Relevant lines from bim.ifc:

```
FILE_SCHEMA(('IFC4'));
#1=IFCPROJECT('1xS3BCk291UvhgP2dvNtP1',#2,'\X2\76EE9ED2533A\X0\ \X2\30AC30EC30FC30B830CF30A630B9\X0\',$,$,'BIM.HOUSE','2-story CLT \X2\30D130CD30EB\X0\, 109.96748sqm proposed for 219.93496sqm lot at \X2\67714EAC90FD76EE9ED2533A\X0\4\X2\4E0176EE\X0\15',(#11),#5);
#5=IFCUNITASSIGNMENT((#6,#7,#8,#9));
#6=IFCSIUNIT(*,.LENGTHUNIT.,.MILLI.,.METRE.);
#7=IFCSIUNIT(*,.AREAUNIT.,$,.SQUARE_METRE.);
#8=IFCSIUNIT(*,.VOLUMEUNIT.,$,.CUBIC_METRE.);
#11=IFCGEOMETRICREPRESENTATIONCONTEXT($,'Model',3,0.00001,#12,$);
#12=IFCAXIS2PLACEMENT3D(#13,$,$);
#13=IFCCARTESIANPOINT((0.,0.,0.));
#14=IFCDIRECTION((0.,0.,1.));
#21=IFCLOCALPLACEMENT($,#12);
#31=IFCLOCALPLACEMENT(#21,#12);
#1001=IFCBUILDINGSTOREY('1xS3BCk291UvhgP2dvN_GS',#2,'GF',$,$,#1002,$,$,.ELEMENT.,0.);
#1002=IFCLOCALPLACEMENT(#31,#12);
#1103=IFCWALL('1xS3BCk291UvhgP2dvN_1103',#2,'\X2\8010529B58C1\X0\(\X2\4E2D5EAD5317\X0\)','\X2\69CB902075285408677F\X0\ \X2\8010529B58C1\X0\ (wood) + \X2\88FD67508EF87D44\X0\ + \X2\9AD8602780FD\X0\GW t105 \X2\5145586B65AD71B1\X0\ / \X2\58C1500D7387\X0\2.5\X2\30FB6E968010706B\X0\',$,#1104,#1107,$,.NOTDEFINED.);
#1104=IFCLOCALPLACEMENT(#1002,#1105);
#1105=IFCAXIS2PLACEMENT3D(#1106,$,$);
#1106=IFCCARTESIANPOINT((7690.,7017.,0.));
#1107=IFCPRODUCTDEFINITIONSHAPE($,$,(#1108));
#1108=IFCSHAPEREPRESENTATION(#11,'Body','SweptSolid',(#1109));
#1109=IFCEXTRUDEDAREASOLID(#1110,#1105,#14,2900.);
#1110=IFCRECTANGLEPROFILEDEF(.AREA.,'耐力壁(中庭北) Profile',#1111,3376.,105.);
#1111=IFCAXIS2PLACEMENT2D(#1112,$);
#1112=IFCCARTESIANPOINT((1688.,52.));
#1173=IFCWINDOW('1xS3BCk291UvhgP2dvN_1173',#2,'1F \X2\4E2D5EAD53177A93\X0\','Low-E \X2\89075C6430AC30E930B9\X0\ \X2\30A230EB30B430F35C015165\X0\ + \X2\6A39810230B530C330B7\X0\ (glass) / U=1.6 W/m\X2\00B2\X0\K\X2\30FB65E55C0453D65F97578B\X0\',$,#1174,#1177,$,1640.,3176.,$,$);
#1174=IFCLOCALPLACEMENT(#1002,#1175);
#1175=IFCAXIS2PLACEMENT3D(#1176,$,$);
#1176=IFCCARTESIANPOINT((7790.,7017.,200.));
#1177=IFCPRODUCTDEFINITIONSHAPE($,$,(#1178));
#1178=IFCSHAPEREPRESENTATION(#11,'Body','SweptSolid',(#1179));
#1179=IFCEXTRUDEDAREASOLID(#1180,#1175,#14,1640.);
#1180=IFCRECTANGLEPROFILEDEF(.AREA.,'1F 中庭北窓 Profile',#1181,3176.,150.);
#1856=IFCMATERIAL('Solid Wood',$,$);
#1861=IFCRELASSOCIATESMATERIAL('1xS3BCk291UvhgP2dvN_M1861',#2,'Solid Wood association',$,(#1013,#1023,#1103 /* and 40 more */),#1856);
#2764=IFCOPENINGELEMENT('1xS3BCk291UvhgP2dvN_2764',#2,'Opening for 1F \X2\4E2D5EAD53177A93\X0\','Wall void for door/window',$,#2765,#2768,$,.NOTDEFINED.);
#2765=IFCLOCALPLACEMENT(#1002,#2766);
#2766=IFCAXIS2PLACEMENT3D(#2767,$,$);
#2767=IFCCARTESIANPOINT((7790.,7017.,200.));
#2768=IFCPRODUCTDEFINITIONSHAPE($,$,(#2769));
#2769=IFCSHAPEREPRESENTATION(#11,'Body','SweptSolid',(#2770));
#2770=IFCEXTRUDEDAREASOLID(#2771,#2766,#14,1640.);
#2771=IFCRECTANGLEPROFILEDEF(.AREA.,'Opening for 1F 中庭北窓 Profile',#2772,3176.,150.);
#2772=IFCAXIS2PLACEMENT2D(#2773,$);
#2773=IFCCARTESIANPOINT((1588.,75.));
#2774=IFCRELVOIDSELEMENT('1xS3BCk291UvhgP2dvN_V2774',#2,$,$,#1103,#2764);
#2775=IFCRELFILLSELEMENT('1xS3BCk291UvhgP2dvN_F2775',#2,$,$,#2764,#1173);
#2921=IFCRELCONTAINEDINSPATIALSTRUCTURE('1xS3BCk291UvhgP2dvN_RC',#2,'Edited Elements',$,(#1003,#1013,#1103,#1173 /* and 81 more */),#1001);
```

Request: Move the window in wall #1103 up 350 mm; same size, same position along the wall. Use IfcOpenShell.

```python
import numpy as np
import ifcopenshell
import ifcopenshell.api.geometry
import ifcopenshell.util.placement
import ifcopenshell.util.unit

model = ifcopenshell.open("bim.ifc")
unit_scale = ifcopenshell.util.unit.calculate_unit_scale(model)

window = model.by_guid("1xS3BCk291UvhgP2dvN_1173")
opening = window.FillsVoids[0].RelatingOpeningElement
dz = 350.0

shift = np.array([0.0, 0.0, dz])
# The window is not placed relative to its opening, so move both.
for product in (opening, window):
    matrix = ifcopenshell.util.placement.get_local_placement(product.ObjectPlacement)
    matrix[:3, 3] += shift
    ifcopenshell.api.geometry.edit_object_placement(model, product=product, matrix=matrix, is_si=False)

print(f"moved by {dz * unit_scale:+.3f} m")

model.write("bim_updated.ifc")
```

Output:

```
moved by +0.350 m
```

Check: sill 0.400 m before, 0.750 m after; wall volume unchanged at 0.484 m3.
